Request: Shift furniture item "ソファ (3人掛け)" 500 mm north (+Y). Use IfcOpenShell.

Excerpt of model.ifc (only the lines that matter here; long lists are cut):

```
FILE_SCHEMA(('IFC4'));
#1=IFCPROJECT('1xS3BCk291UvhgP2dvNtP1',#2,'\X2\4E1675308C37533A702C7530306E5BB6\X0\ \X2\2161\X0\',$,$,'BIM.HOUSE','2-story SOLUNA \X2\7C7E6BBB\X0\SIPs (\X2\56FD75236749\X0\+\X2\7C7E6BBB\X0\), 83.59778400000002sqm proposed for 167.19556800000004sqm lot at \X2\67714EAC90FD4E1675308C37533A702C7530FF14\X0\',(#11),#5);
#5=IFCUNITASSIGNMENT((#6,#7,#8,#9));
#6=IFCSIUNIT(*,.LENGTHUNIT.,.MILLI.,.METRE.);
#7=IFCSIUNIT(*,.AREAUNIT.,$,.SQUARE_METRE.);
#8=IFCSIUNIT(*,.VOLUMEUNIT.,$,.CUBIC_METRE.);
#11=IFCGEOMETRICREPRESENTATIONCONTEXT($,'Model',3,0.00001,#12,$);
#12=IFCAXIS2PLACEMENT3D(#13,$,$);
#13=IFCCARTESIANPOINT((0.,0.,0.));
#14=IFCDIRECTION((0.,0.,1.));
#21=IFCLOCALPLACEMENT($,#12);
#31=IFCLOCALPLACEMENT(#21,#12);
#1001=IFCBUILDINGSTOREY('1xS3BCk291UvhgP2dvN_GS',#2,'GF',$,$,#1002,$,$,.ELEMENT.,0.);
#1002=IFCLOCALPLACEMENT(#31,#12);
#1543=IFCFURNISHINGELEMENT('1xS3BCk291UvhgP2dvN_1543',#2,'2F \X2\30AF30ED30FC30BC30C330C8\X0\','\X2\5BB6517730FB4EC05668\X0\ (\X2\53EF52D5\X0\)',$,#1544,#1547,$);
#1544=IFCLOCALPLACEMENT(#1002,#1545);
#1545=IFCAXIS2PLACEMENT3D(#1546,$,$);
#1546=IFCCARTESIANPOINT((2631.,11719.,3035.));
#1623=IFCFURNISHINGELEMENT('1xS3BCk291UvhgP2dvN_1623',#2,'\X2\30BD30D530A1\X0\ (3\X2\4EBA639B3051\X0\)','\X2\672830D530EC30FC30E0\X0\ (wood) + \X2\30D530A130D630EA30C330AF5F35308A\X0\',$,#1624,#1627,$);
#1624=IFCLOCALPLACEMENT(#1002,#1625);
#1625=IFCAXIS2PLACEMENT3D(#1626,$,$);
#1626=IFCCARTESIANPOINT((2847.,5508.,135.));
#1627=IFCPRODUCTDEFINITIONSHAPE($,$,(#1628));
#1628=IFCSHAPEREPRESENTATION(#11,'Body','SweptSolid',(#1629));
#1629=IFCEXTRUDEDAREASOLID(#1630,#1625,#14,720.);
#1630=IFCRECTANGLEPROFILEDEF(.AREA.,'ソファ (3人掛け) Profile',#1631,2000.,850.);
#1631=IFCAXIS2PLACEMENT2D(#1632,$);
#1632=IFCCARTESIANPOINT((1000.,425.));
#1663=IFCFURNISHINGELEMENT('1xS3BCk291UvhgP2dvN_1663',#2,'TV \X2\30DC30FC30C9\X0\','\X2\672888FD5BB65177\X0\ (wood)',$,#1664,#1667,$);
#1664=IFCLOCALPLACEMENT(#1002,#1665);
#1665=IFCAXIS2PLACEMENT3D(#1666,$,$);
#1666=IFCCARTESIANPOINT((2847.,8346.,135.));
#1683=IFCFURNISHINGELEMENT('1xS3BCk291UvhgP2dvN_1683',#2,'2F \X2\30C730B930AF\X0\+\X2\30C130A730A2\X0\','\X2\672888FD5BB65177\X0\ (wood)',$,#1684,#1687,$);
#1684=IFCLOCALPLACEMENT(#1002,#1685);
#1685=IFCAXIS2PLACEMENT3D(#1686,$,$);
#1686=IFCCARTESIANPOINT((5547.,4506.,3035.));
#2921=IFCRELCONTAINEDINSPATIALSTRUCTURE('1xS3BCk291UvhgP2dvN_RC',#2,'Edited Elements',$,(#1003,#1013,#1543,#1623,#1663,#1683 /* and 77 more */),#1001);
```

```python
import ifcopenshell
import ifcopenshell.api.geometry
import ifcopenshell.util.placement
import ifcopenshell.util.unit

model = ifcopenshell.open("model.ifc")
unit_scale = ifcopenshell.util.unit.calculate_unit_scale(model)

item = model.by_id(1623)
matrix = ifcopenshell.util.placement.get_local_placement(item.ObjectPlacement)
matrix[1, 3] += 0.5 / unit_scale
ifcopenshell.api.geometry.edit_object_placement(model, product=item, matrix=matrix, is_si=False)

print(ifcopenshell.util.placement.get_local_placement(item.ObjectPlacement).round(3) + 0.0)

model.write("model_v2.ifc")
```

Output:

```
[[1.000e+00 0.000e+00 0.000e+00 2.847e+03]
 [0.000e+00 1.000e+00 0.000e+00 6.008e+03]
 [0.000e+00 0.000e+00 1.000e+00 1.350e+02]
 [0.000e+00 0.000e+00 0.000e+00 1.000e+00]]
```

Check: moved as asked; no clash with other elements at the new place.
